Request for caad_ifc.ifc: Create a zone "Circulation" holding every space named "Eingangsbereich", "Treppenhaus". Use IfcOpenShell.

First a look at what the model holds.

```python
import ifcopenshell

model = ifcopenshell.open("caad_ifc.ifc")
print(model.schema)
seen = {}
for space in model.by_type("IfcSpace"):
    seen[space.LongName] = seen.get(space.LongName, 0) + 1
for name, count in sorted(seen.items(), key=str):
    print(count, "x", name)
print("zones:", [z.Name for z in model.by_type("IfcZone")][:20])
```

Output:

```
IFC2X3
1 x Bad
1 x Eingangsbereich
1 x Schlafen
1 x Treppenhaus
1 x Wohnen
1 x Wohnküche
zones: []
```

```python
import ifcopenshell
import ifcopenshell.api.group
import ifcopenshell.api.root

model = ifcopenshell.open("caad_ifc.ifc")

names = {"Eingangsbereich", "Treppenhaus"}
spaces = [s for s in model.by_type("IfcSpace") if s.LongName in names]

zone = ifcopenshell.api.root.create_entity(model, ifc_class="IfcZone", name="Circulation")
ifcopenshell.api.group.assign_group(model, products=spaces, group=zone)
print(len(spaces), "spaces in", zone.Name)

model.write("caad_ifc_edited.ifc")
```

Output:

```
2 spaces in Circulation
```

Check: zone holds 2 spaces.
